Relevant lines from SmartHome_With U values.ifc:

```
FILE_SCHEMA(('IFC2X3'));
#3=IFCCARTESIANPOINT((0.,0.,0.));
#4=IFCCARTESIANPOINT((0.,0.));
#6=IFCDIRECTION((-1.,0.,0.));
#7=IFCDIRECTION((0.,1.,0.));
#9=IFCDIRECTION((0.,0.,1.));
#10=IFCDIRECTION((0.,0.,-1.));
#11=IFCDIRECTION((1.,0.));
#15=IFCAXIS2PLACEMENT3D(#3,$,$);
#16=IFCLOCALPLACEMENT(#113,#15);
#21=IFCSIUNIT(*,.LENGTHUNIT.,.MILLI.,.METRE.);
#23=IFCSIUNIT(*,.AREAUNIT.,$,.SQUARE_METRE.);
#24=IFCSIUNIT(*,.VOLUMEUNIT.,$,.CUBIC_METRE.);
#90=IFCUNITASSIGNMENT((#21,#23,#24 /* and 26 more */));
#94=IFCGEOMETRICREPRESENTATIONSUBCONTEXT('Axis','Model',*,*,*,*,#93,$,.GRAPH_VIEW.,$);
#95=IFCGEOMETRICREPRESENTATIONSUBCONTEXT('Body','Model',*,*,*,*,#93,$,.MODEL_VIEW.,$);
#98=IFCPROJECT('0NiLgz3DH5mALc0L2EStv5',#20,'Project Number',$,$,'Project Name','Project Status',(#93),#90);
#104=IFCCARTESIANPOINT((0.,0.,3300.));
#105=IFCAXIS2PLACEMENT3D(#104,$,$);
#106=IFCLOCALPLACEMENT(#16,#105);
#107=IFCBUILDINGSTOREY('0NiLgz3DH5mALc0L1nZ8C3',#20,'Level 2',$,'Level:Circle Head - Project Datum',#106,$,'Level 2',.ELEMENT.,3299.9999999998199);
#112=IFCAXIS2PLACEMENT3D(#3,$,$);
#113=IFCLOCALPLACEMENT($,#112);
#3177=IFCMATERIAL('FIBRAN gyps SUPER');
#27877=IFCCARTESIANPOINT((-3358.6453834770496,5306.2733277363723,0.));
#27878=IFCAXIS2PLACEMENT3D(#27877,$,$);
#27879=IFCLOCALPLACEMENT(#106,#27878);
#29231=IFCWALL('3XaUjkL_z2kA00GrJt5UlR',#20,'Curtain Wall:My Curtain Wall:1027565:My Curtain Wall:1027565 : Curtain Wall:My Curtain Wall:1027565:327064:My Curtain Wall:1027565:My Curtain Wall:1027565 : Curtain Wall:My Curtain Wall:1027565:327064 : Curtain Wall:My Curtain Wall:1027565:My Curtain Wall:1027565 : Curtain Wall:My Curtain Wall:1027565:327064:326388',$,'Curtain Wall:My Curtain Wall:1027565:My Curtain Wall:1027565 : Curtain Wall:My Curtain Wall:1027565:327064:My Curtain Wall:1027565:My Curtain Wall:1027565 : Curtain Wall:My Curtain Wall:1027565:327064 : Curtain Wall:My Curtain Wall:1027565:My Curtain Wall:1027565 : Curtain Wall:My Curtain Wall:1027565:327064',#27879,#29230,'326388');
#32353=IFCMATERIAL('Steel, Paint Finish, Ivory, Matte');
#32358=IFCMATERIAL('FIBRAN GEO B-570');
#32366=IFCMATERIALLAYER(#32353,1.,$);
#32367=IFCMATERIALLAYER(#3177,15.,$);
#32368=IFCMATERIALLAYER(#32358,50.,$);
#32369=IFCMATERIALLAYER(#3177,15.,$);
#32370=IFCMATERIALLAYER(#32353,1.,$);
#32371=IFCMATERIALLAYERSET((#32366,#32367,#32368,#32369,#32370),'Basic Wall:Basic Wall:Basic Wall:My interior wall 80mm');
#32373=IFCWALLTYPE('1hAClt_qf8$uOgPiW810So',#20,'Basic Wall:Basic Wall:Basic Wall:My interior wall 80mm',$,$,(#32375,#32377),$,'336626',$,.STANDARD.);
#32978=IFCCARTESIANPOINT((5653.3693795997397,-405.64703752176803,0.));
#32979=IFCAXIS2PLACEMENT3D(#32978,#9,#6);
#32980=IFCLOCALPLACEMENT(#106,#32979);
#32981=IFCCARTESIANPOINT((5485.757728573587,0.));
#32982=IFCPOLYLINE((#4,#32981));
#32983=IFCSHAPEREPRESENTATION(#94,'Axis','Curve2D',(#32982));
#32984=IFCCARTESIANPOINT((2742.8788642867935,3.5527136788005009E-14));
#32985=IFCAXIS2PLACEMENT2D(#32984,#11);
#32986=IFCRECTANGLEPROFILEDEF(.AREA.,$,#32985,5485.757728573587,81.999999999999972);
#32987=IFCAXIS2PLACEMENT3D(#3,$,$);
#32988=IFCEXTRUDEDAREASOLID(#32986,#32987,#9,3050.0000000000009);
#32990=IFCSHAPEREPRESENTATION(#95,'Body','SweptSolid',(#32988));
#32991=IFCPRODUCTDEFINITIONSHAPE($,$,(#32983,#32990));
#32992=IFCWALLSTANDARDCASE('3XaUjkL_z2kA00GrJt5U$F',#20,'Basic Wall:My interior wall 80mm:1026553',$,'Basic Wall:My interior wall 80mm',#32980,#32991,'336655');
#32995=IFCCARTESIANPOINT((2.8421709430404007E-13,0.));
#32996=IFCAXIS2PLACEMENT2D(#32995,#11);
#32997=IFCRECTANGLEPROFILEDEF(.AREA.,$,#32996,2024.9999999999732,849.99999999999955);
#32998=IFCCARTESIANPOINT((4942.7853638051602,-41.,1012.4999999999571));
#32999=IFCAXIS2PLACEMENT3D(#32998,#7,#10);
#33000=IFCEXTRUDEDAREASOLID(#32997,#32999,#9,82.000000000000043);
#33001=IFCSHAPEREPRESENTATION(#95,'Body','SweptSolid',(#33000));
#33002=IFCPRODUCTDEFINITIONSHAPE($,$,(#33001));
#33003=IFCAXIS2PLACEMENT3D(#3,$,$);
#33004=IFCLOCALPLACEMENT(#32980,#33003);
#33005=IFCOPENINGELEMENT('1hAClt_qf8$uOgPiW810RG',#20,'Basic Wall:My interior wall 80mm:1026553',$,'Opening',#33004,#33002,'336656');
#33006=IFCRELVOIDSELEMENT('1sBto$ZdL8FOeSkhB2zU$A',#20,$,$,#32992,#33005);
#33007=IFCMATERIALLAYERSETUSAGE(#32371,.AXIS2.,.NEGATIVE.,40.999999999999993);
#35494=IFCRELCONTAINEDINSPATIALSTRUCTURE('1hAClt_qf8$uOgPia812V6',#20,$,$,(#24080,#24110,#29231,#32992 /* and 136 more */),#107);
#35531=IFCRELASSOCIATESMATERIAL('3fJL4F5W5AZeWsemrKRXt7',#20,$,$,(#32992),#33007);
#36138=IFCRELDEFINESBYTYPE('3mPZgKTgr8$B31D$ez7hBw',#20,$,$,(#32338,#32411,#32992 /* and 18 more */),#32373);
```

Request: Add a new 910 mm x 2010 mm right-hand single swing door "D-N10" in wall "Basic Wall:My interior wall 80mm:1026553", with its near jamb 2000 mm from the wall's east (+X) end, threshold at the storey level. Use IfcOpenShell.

```python
import numpy as np
import ifcopenshell
import ifcopenshell.api.feature
import ifcopenshell.api.geometry
import ifcopenshell.api.root
import ifcopenshell.api.spatial
import ifcopenshell.api.type
import ifcopenshell.geom
import ifcopenshell.util.element
import ifcopenshell.util.placement
import ifcopenshell.util.representation
import ifcopenshell.util.shape
import ifcopenshell.util.unit

model = ifcopenshell.open("SmartHome_With U values.ifc")
unit_scale = ifcopenshell.util.unit.calculate_unit_scale(model)
settings = ifcopenshell.geom.settings()


def volume(element):
    """Net volume in cubic metres, openings subtracted."""
    shape = ifcopenshell.geom.create_shape(settings, element)
    return ifcopenshell.util.shape.get_volume(shape.geometry)


wall = model.by_guid("3XaUjkL_z2kA00GrJt5U$F")
storey = ifcopenshell.util.element.get_container(wall, ifc_class="IfcBuildingStorey")
context = ifcopenshell.util.representation.get_context(model, "Model", "Body", "MODEL_VIEW")
before = volume(wall)

width, height, from_end, sill = 0.91, 2.01, 2, 0.0  # metres

# The wall runs along its own X axis, and the end named is its -X end.
wall_shape = ifcopenshell.geom.create_shape(settings, wall)
x, y, z = ifcopenshell.util.shape.get_vertices(wall_shape.geometry).T
start = x.min() + from_end
face, thickness = float(y.min()), float(y.max() - y.min())
wall_matrix = ifcopenshell.util.placement.get_local_placement(wall.ObjectPlacement)
level = ifcopenshell.util.placement.get_local_placement(storey.ObjectPlacement)[2, 3]


def in_wall(x, y):
    """Placement at x, y metres in the wall's axes, at sill height."""
    matrix = wall_matrix.copy()
    matrix[:, 3] = wall_matrix @ np.array([x / unit_scale, y / unit_scale, 0.0, 1.0])
    matrix[2, 3] = level + sill / unit_scale
    return matrix


# Opening: a box that overshoots both wall faces by 50 mm.
opening = ifcopenshell.api.root.create_entity(model, ifc_class="IfcOpeningElement")
box = ifcopenshell.api.geometry.add_wall_representation(
    model, context=context, length=width, height=height, thickness=thickness + 0.1
)
ifcopenshell.api.geometry.assign_representation(model, product=opening, representation=box)
ifcopenshell.api.geometry.edit_object_placement(model, product=opening, matrix=in_wall(start, face - 0.05), is_si=False)
ifcopenshell.api.feature.add_feature(model, feature=opening, element=wall)

door = ifcopenshell.api.root.create_entity(model, ifc_class="IfcDoor", name="D-N10")
door.OverallWidth, door.OverallHeight = width / unit_scale, height / unit_scale
body = ifcopenshell.api.geometry.add_door_representation(
    model,
    context=context,
    overall_width=door.OverallWidth,
    overall_height=door.OverallHeight,
    operation_type="SINGLE_SWING_RIGHT",
    lining_properties={"LiningDepth": thickness / unit_scale, "ThresholdDepth": thickness / unit_scale},
)
ifcopenshell.api.geometry.assign_representation(model, product=door, representation=body)
ifcopenshell.api.spatial.assign_container(model, products=[door], relating_structure=storey)
fills = ifcopenshell.api.feature.add_filling(model, opening=opening, element=door)
fills.OwnerHistory = door.OwnerHistory  # required in IFC2X3

# IFC2X3 keeps the operation on the door style.
style = ifcopenshell.api.root.create_entity(model, ifc_class="IfcDoorStyle", name="D-N10")
style.OperationType, style.ConstructionType = "SINGLE_SWING_RIGHT", "NOTDEFINED"
style.ParameterTakesPrecedence = style.Sizeable = False
ifcopenshell.api.type.assign_type(model, related_objects=[door], relating_type=style)

# The lining spans the wall, so the door starts at the wall face.
ifcopenshell.api.geometry.edit_object_placement(model, product=door, matrix=in_wall(start, face), is_si=False)

after = volume(wall)

print(f"wall volume {before:.3f} -> {after:.3f} m3")

model.write("SmartHome_With U values_v2.ifc")
```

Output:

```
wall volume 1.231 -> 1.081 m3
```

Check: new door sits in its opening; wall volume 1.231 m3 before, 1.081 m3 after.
